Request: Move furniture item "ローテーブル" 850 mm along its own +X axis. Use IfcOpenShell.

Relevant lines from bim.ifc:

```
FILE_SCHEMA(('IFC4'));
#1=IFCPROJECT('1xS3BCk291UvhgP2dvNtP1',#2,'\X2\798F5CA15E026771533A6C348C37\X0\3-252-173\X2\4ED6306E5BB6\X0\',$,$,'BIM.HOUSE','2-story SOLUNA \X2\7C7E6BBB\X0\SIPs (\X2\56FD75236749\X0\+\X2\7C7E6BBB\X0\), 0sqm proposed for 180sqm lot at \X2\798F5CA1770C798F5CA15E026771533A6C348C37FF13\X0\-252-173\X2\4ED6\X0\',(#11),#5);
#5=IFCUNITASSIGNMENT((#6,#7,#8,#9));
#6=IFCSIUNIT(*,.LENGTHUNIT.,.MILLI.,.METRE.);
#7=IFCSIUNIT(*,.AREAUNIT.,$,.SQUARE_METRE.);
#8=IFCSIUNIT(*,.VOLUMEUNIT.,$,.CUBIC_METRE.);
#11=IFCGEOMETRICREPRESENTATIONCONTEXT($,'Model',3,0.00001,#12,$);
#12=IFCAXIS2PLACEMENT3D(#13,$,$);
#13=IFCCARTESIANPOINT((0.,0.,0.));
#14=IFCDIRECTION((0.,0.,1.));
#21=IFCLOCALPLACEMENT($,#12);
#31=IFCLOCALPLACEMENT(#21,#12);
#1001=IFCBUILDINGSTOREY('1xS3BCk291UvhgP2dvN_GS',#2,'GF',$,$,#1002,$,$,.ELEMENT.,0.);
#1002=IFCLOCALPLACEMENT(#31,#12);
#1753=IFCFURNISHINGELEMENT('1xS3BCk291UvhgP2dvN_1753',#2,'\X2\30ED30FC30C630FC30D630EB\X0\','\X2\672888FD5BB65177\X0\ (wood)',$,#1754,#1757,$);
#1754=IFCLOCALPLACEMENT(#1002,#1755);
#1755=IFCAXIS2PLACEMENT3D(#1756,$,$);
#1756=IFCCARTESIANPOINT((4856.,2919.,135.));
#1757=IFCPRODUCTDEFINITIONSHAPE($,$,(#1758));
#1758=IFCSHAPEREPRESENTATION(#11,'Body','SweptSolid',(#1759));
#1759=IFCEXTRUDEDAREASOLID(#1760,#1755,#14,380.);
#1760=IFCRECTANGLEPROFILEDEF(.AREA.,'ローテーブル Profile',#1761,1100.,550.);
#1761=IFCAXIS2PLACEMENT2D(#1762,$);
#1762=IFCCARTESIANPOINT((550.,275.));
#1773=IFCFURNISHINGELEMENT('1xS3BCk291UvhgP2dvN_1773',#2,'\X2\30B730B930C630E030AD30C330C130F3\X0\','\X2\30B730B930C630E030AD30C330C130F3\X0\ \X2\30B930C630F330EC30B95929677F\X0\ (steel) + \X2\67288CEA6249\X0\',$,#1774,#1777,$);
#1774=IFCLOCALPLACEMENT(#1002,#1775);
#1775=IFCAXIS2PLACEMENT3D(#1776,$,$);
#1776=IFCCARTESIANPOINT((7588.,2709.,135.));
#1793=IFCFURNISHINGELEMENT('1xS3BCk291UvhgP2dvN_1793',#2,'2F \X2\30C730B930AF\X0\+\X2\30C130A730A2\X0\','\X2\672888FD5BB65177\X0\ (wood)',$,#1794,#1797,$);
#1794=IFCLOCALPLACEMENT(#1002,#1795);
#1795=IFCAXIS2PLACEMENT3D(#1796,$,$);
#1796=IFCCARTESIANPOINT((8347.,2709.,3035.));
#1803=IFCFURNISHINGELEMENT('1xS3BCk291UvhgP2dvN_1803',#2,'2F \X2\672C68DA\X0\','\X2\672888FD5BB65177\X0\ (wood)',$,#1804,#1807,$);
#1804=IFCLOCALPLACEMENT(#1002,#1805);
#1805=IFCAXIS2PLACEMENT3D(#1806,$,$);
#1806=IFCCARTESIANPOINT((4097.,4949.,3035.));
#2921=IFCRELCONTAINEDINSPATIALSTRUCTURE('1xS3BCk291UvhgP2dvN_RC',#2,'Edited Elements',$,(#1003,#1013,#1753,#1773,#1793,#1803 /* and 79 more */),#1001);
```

```python
import ifcopenshell
import ifcopenshell.api.geometry
import ifcopenshell.util.placement

model = ifcopenshell.open("bim.ifc")

item = model.by_guid("1xS3BCk291UvhgP2dvN_1753")
matrix = ifcopenshell.util.placement.get_local_placement(item.ObjectPlacement)
matrix[:3, 3] += matrix[:3, 0] * 850.0
ifcopenshell.api.geometry.edit_object_placement(model, product=item, matrix=matrix, is_si=False)

print(ifcopenshell.util.placement.get_local_placement(item.ObjectPlacement).round(3) + 0.0)

model.write("bim_edited.ifc")
```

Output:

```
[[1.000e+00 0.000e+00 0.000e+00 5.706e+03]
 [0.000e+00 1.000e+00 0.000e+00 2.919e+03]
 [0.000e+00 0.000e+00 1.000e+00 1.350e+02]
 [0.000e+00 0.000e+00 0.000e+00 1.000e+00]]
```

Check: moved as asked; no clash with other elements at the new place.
